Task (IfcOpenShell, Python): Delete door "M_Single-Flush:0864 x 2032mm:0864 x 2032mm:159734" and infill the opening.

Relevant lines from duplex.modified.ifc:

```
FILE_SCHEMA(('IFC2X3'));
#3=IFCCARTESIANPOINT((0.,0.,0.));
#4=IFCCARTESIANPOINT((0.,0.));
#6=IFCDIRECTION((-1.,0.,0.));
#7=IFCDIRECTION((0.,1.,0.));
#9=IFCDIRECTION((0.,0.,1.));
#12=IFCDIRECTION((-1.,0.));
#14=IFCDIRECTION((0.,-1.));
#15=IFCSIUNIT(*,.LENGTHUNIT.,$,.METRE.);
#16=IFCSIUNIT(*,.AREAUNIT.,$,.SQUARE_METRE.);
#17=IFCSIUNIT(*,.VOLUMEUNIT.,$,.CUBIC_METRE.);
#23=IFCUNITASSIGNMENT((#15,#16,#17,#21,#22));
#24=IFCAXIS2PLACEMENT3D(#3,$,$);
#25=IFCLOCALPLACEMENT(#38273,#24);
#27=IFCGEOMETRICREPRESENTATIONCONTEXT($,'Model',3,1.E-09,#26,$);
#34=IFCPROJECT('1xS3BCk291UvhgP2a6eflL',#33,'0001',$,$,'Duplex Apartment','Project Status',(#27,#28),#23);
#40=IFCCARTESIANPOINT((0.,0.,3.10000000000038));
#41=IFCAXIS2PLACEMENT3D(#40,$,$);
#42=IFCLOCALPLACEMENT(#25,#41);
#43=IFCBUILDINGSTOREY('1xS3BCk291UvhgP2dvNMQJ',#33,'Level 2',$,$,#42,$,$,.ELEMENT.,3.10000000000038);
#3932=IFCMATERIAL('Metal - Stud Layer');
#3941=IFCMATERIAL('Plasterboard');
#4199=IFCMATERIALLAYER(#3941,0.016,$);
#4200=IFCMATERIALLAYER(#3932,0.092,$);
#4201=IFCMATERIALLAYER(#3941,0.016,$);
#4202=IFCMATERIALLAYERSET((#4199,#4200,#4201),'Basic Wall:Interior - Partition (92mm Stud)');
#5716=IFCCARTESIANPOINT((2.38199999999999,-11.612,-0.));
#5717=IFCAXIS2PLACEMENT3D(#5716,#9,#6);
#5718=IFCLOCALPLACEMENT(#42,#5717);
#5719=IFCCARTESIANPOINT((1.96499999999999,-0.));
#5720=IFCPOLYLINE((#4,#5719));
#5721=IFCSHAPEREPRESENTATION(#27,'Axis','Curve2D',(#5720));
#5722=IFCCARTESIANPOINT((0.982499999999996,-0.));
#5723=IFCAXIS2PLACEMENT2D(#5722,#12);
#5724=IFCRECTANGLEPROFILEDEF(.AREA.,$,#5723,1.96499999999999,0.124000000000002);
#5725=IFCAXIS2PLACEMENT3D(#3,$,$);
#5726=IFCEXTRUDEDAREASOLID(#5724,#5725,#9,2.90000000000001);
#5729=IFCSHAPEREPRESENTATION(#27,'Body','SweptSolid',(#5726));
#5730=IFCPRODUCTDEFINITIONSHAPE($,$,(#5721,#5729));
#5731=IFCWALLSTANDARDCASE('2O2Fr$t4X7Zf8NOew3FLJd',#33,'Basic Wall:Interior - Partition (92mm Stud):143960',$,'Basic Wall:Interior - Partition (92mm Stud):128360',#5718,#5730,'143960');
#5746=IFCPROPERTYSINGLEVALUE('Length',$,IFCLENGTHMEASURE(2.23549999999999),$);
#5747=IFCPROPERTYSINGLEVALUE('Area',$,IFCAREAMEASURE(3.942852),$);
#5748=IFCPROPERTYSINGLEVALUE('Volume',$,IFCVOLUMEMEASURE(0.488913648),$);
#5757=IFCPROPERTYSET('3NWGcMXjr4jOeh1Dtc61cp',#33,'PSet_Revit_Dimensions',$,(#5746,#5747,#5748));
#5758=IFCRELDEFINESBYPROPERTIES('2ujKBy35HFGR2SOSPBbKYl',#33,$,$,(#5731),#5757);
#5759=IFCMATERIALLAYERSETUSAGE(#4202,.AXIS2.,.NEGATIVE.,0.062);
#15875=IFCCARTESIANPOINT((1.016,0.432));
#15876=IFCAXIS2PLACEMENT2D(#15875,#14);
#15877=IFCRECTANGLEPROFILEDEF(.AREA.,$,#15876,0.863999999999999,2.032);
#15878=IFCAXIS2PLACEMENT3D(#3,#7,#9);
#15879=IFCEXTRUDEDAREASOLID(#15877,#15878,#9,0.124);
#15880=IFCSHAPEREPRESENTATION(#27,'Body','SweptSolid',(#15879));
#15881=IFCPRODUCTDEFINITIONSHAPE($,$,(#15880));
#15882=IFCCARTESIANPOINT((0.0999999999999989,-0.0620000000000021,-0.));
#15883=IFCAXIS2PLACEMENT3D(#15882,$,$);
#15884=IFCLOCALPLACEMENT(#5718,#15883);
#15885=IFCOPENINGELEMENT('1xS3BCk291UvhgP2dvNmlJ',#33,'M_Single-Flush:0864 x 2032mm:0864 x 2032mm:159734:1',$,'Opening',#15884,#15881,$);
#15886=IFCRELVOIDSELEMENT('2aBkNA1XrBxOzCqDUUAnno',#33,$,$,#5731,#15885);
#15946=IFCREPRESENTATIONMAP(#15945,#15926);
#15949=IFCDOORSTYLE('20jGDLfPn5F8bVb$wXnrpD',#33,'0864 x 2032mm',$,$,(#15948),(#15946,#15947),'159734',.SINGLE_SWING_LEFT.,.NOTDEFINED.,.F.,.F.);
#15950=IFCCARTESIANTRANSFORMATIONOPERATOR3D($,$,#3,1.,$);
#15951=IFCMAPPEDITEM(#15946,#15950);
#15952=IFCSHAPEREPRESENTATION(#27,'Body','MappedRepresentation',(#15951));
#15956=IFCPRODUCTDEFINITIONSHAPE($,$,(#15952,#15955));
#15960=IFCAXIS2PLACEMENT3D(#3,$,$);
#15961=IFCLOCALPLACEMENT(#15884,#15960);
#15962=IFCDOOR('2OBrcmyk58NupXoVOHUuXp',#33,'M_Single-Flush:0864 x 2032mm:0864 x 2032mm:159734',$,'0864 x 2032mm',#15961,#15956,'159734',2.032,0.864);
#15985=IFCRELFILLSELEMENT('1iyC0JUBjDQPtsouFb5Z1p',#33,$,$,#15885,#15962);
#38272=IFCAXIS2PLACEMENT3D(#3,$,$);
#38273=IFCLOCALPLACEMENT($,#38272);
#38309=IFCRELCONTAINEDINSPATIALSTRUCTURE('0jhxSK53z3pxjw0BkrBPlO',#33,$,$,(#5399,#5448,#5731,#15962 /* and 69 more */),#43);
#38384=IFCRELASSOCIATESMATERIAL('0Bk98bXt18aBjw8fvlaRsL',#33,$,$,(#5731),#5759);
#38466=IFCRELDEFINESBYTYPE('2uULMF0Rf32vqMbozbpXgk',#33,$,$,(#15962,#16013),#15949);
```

```python
import ifcopenshell
import ifcopenshell.api.feature
import ifcopenshell.api.pset
import ifcopenshell.api.root
import ifcopenshell.geom
import ifcopenshell.util.element
import ifcopenshell.util.shape
import ifcopenshell.util.unit

model = ifcopenshell.open("duplex.modified.ifc")
area_scale = ifcopenshell.util.unit.calculate_unit_scale(model, "AREAUNIT")
volume_scale = ifcopenshell.util.unit.calculate_unit_scale(model, "VOLUMEUNIT")
settings = ifcopenshell.geom.settings()


def volume(element):
    """Net volume in cubic metres, openings subtracted."""
    shape = ifcopenshell.geom.create_shape(settings, element)
    return ifcopenshell.util.shape.get_volume(shape.geometry)


door = model.by_id(15962)
opening = door.FillsVoids[0].RelatingOpeningElement
wall = opening.VoidsElements[0].RelatingBuildingElement
before = volume(wall)

ifcopenshell.api.root.remove_product(model, product=door)
ifcopenshell.api.feature.remove_feature(model, feature=opening)

after = volume(wall)
thickness = 0.124  # wall thickness in metres

# Update the wall's stored quantities.
pset = model.by_id(ifcopenshell.util.element.get_pset(wall, "PSet_Revit_Dimensions", should_inherit=False)["id"])
ifcopenshell.api.pset.edit_pset(model, pset=pset, properties={
    "Area": model.create_entity("IfcAreaMeasure", after / thickness / area_scale),
    "Volume": model.create_entity("IfcVolumeMeasure", after / volume_scale),
})

print(f"wall volume {before:.3f} -> {after:.3f} m3")

model.write("duplex.modified_updated.ifc")
```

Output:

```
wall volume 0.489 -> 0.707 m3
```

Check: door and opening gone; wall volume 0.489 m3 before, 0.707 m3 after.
